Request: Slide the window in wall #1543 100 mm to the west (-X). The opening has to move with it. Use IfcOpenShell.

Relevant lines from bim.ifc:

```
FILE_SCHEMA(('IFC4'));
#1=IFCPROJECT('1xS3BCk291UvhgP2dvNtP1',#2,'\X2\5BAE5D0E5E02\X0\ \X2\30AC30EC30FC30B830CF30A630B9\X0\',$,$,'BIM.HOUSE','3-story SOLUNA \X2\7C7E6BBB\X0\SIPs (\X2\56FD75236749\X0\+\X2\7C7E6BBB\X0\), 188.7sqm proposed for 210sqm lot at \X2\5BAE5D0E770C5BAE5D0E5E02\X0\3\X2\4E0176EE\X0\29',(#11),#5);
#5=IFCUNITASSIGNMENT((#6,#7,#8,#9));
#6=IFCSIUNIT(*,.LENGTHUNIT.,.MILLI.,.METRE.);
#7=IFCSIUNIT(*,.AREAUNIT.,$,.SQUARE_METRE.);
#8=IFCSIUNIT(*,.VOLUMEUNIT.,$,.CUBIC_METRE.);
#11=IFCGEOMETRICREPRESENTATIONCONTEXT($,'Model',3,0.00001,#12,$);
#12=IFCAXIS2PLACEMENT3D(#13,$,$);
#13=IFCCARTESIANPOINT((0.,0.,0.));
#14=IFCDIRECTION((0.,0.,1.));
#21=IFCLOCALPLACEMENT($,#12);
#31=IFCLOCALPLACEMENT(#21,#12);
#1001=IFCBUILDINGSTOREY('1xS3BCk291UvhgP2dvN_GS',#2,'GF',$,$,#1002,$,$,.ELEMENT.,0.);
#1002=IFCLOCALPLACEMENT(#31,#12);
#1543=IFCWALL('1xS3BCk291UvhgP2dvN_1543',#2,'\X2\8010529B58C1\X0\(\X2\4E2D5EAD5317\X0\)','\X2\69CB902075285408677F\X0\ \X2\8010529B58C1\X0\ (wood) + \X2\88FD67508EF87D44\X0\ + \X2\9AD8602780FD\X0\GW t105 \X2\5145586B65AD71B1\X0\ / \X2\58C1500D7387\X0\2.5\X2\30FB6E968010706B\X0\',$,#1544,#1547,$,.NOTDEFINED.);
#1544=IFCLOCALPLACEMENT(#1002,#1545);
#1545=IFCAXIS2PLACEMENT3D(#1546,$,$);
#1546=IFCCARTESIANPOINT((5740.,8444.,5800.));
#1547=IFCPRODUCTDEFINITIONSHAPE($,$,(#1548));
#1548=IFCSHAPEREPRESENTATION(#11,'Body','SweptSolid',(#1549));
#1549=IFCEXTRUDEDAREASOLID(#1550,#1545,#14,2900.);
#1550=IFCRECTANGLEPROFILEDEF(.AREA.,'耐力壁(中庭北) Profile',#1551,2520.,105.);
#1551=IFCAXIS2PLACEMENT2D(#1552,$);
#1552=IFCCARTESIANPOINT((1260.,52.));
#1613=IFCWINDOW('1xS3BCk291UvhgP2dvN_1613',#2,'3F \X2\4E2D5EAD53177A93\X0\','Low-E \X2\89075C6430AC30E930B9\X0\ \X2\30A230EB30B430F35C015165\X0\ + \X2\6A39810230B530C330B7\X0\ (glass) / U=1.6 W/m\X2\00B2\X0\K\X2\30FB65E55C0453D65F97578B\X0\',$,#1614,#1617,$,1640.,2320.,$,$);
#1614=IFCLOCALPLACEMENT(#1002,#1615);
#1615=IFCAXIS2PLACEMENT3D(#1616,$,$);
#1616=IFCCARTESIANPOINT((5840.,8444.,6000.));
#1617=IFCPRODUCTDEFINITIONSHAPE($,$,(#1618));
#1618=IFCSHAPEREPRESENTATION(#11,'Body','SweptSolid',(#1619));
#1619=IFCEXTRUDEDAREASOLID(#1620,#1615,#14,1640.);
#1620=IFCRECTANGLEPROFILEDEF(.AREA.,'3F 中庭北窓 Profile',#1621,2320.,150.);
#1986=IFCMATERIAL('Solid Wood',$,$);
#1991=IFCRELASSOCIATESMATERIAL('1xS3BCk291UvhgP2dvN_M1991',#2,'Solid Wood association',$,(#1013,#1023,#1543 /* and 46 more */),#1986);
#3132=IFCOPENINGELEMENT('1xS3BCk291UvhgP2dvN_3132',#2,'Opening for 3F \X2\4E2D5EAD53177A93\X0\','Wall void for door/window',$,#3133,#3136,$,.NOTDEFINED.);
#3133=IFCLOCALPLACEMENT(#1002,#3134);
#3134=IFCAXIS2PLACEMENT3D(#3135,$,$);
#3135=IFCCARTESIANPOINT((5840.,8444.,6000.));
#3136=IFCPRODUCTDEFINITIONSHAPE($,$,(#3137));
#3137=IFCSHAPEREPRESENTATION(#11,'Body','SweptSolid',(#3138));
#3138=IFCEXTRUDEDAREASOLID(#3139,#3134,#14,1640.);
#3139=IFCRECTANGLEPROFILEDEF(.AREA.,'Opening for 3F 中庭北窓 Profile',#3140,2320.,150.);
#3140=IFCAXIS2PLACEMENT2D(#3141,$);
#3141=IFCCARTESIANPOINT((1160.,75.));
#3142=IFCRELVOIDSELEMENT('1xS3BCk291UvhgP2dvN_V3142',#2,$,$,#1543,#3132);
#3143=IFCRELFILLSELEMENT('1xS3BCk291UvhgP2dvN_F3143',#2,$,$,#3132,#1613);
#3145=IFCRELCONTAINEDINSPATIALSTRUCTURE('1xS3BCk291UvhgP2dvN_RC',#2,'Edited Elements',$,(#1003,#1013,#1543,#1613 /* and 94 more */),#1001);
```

```python
import ifcopenshell
import ifcopenshell.api.geometry
import ifcopenshell.util.placement

model = ifcopenshell.open("bim.ifc")

window = model.by_guid("1xS3BCk291UvhgP2dvN_1613")
opening = window.FillsVoids[0].RelatingOpeningElement
wall = opening.VoidsElements[0].RelatingBuildingElement

wall_matrix = ifcopenshell.util.placement.get_local_placement(wall.ObjectPlacement)
shift = wall_matrix[:3, 0] * -100.0
before = ifcopenshell.util.placement.get_local_placement(window.ObjectPlacement)[:3, 3].copy()

# The window is not placed relative to its opening, so move both.
for product in (opening, window):
    matrix = ifcopenshell.util.placement.get_local_placement(product.ObjectPlacement)
    matrix[:3, 3] += shift
    ifcopenshell.api.geometry.edit_object_placement(model, product=product, matrix=matrix, is_si=False)

after = ifcopenshell.util.placement.get_local_placement(window.ObjectPlacement)[:3, 3]
print("window moved by", (after - before).round(3) + 0.0)

model.write("bim_updated.ifc")
```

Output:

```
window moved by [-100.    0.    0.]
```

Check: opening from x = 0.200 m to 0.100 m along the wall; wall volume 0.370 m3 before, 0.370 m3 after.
